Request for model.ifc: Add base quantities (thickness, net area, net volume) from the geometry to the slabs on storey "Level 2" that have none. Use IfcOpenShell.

First a look at what the model holds.

```python
import ifcopenshell
import ifcopenshell.util.element
import ifcopenshell.util.unit

model = ifcopenshell.open("model.ifc")
print(model.schema)
for unit_type in ("LENGTHUNIT", "AREAUNIT", "VOLUMEUNIT"):
    print(unit_type, ifcopenshell.util.unit.calculate_unit_scale(model, unit_type))
storey = next(s for s in model.by_type("IfcBuildingStorey") if s.Name == "Level 2")
slabs = [e for e in ifcopenshell.util.element.get_decomposition(storey) if e.is_a("IfcSlab")]
for e in sorted(slabs, key=lambda e: e.id()):
    print(e.id(), e.is_a(), e.Name, list(ifcopenshell.util.element.get_psets(e, qtos_only=True)), sep=" | ")
```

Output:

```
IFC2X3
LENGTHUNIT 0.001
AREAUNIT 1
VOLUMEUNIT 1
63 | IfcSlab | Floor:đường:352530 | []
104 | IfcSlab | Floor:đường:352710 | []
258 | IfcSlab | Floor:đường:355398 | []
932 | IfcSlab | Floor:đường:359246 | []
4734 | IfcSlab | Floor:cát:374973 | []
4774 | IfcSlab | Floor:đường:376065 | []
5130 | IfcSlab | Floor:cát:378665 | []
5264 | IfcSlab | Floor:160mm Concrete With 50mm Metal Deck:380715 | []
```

```python
import ifcopenshell
import ifcopenshell.api.pset
import ifcopenshell.geom
import ifcopenshell.util.element
import ifcopenshell.util.shape
import ifcopenshell.util.unit

model = ifcopenshell.open("model.ifc")
unit_scale = ifcopenshell.util.unit.calculate_unit_scale(model)
area_scale = ifcopenshell.util.unit.calculate_unit_scale(model, "AREAUNIT")
volume_scale = ifcopenshell.util.unit.calculate_unit_scale(model, "VOLUMEUNIT")
settings = ifcopenshell.geom.settings()

storey = next(s for s in model.by_type("IfcBuildingStorey") if s.Name == "Level 2")
slabs = [e for e in ifcopenshell.util.element.get_decomposition(storey) if e.is_a("IfcSlab")]

for e in sorted(slabs, key=lambda e: e.id()):
    if ifcopenshell.util.element.get_psets(e, qtos_only=True, should_inherit=False):
        continue
    # Geometry comes back in metres, in the element's own axes.
    shape = ifcopenshell.geom.create_shape(settings, e)
    values = {
        "Width": ifcopenshell.util.shape.get_z(shape.geometry) / unit_scale,
        "NetArea": ifcopenshell.util.shape.get_footprint_area(shape.geometry) / area_scale,
        "NetVolume": ifcopenshell.util.shape.get_volume(shape.geometry) / volume_scale,
    }
    qto = ifcopenshell.api.pset.add_qto(model, product=e, name="BaseQuantities")
    ifcopenshell.api.pset.edit_qto(model, qto=qto, properties=values)
    print(e.id(), {k: round(v, 3) for k, v in values.items()})

model.write("model-out.ifc")
```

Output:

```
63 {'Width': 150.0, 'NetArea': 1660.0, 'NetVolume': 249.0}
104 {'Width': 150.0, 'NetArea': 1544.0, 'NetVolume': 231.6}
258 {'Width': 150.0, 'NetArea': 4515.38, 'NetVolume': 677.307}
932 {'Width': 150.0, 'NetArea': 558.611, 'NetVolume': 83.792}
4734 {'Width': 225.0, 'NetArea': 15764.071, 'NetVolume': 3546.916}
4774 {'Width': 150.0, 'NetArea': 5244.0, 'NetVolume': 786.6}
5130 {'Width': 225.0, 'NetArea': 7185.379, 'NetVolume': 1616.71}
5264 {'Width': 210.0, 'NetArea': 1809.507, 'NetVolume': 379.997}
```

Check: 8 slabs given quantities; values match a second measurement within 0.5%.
